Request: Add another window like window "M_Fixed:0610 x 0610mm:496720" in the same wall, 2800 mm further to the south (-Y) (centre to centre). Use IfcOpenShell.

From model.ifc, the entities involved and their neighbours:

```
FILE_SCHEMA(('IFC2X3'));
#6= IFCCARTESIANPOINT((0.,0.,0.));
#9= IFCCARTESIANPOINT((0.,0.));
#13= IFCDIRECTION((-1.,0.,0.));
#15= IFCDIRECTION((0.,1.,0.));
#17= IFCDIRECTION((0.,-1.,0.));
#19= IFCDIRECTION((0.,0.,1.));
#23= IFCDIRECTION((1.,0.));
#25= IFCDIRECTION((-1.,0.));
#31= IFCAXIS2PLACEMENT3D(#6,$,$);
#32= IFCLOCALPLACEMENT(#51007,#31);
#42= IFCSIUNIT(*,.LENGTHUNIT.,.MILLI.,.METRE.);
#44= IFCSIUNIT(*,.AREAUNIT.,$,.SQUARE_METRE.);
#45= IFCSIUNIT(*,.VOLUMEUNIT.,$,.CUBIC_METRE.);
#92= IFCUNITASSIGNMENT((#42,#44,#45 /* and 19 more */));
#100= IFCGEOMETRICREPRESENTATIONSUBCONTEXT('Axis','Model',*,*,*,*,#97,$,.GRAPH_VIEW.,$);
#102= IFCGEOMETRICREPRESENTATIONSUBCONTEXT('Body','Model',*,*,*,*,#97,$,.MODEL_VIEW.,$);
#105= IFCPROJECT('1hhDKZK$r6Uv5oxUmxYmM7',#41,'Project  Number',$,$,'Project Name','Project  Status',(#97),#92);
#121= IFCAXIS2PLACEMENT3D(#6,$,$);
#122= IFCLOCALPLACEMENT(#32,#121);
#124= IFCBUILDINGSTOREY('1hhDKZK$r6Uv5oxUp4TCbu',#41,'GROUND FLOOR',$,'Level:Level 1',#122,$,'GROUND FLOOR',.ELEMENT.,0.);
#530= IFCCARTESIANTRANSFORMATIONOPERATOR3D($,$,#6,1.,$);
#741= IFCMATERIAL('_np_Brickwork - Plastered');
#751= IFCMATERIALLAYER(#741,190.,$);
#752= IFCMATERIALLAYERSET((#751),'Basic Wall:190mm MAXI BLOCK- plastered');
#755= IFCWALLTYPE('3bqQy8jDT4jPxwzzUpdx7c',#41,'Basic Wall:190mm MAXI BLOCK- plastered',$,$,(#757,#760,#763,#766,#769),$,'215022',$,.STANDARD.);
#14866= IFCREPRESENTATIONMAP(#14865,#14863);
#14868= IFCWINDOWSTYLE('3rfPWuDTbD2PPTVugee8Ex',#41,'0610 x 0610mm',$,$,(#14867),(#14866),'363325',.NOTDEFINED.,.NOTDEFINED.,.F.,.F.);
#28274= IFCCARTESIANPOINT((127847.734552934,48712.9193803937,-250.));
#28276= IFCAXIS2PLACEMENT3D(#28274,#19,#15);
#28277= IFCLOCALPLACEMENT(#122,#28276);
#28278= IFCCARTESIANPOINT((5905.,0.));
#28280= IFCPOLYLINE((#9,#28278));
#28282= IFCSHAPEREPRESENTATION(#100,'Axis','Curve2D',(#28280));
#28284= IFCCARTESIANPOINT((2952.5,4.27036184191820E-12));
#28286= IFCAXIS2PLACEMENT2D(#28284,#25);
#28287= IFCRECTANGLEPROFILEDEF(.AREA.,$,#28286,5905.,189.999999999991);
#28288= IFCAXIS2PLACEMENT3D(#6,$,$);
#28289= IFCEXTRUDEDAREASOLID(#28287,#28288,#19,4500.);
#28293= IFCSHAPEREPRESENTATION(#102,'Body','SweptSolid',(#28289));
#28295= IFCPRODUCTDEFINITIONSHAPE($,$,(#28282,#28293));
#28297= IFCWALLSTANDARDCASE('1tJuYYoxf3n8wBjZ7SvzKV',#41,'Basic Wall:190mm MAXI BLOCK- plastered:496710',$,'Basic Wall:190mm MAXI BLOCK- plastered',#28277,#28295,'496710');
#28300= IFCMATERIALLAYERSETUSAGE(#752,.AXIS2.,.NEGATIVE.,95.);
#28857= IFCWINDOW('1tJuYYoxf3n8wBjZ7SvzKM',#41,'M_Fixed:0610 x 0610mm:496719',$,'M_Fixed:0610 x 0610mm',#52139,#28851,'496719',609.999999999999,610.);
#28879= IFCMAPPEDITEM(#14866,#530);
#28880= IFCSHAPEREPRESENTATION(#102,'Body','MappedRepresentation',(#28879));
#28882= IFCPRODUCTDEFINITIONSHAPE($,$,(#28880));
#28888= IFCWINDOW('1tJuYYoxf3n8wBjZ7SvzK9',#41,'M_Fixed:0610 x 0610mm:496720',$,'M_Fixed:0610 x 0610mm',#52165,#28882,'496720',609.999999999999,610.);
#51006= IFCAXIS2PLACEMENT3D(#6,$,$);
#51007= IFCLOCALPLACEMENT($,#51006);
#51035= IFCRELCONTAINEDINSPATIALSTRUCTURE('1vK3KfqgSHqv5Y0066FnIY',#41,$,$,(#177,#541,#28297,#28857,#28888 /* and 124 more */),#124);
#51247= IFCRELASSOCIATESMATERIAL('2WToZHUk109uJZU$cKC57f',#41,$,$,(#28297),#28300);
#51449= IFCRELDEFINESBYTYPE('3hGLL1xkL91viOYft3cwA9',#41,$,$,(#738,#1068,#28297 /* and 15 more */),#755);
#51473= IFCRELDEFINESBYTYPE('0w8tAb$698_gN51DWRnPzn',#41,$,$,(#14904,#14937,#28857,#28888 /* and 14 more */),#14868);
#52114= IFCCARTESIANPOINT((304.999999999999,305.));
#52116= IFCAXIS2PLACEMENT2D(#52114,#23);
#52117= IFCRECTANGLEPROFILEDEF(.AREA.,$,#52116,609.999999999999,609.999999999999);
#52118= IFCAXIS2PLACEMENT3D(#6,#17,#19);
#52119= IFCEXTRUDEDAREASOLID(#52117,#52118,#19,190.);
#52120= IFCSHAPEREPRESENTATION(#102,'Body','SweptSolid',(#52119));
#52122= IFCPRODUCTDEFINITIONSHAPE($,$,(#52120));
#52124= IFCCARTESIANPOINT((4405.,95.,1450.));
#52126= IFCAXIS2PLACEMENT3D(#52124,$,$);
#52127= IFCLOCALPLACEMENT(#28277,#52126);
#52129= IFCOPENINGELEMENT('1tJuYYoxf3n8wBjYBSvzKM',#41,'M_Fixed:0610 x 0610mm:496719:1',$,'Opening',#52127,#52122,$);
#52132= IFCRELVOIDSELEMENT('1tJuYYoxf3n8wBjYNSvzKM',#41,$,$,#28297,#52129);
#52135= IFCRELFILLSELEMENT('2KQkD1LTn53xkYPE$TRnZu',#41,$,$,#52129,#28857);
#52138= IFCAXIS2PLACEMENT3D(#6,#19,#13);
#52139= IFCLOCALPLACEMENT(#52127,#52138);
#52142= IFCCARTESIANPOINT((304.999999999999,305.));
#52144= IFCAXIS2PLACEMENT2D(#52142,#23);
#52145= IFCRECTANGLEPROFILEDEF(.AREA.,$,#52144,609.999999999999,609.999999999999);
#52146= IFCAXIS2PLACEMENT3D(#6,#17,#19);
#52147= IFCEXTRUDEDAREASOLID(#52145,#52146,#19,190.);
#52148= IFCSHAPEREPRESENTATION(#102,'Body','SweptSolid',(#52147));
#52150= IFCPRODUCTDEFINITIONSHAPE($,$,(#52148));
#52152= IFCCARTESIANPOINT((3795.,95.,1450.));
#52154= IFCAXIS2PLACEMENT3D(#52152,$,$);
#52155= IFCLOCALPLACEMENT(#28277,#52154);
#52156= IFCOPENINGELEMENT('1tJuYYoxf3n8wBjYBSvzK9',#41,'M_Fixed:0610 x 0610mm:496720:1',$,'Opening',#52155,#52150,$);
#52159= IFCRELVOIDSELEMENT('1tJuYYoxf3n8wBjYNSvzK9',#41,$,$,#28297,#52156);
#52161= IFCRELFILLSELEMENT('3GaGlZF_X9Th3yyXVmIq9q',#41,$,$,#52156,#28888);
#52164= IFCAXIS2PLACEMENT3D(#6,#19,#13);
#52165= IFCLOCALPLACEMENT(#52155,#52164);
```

```python
import ifcopenshell
import ifcopenshell.api.feature
import ifcopenshell.api.geometry
import ifcopenshell.api.root
import ifcopenshell.geom
import ifcopenshell.util.element
import ifcopenshell.util.placement
import ifcopenshell.util.shape
import ifcopenshell.util.unit

model = ifcopenshell.open("model.ifc")
unit_scale = ifcopenshell.util.unit.calculate_unit_scale(model)
settings = ifcopenshell.geom.settings()


def volume(element):
    """Net volume in cubic metres, openings subtracted."""
    shape = ifcopenshell.geom.create_shape(settings, element)
    return ifcopenshell.util.shape.get_volume(shape.geometry)


def reuse_history(source, copy):
    """copy_class also copies each property set's owner history, people and application; keep the originals."""
    for rel in copy.IsDefinedBy:
        if rel.is_a("IfcRelDefinesByProperties") and (history := rel.RelatingPropertyDefinition.OwnerHistory):
            rel.RelatingPropertyDefinition.OwnerHistory = source.OwnerHistory
            ifcopenshell.util.element.remove_deep2(model, history)


window = model.by_guid("1tJuYYoxf3n8wBjZ7SvzK9")
opening = window.FillsVoids[0].RelatingOpeningElement
wall = opening.VoidsElements[0].RelatingBuildingElement
before = volume(wall)
shift = ifcopenshell.util.placement.get_local_placement(wall.ObjectPlacement)[:3, 0] * -2.8 / unit_scale

# copy_class copies the void relationship, type, container and properties, but no geometry.
new_opening = ifcopenshell.api.root.copy_class(model, product=opening)
new_opening.Representation = ifcopenshell.util.element.copy_deep(
    model, opening.Representation, exclude=["IfcGeometricRepresentationContext", "IfcRepresentationMap"]
)
new_opening.Name = "M_Fixed:0610 x 0610mm"
new_window = ifcopenshell.api.root.copy_class(model, product=window)
new_window.Representation = ifcopenshell.util.element.copy_deep(
    model, window.Representation, exclude=["IfcGeometricRepresentationContext", "IfcRepresentationMap"]
)
new_window.Name = "M_Fixed:0610 x 0610mm"
new_window.Tag = None
reuse_history(window, new_window)
fills = ifcopenshell.api.feature.add_filling(model, opening=new_opening, element=new_window)
fills.OwnerHistory = new_window.OwnerHistory  # required in IFC2X3

for old, new in ((opening, new_opening), (window, new_window)):
    matrix = ifcopenshell.util.placement.get_local_placement(old.ObjectPlacement)
    matrix[:3, 3] += shift
    ifcopenshell.api.geometry.edit_object_placement(model, product=new, matrix=matrix, is_si=False)

after = volume(wall)

print(f"wall volume {before:.3f} -> {after:.3f} m3")

model.write("model-out.ifc")
```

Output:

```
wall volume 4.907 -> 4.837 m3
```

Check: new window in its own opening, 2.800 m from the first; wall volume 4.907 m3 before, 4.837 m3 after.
